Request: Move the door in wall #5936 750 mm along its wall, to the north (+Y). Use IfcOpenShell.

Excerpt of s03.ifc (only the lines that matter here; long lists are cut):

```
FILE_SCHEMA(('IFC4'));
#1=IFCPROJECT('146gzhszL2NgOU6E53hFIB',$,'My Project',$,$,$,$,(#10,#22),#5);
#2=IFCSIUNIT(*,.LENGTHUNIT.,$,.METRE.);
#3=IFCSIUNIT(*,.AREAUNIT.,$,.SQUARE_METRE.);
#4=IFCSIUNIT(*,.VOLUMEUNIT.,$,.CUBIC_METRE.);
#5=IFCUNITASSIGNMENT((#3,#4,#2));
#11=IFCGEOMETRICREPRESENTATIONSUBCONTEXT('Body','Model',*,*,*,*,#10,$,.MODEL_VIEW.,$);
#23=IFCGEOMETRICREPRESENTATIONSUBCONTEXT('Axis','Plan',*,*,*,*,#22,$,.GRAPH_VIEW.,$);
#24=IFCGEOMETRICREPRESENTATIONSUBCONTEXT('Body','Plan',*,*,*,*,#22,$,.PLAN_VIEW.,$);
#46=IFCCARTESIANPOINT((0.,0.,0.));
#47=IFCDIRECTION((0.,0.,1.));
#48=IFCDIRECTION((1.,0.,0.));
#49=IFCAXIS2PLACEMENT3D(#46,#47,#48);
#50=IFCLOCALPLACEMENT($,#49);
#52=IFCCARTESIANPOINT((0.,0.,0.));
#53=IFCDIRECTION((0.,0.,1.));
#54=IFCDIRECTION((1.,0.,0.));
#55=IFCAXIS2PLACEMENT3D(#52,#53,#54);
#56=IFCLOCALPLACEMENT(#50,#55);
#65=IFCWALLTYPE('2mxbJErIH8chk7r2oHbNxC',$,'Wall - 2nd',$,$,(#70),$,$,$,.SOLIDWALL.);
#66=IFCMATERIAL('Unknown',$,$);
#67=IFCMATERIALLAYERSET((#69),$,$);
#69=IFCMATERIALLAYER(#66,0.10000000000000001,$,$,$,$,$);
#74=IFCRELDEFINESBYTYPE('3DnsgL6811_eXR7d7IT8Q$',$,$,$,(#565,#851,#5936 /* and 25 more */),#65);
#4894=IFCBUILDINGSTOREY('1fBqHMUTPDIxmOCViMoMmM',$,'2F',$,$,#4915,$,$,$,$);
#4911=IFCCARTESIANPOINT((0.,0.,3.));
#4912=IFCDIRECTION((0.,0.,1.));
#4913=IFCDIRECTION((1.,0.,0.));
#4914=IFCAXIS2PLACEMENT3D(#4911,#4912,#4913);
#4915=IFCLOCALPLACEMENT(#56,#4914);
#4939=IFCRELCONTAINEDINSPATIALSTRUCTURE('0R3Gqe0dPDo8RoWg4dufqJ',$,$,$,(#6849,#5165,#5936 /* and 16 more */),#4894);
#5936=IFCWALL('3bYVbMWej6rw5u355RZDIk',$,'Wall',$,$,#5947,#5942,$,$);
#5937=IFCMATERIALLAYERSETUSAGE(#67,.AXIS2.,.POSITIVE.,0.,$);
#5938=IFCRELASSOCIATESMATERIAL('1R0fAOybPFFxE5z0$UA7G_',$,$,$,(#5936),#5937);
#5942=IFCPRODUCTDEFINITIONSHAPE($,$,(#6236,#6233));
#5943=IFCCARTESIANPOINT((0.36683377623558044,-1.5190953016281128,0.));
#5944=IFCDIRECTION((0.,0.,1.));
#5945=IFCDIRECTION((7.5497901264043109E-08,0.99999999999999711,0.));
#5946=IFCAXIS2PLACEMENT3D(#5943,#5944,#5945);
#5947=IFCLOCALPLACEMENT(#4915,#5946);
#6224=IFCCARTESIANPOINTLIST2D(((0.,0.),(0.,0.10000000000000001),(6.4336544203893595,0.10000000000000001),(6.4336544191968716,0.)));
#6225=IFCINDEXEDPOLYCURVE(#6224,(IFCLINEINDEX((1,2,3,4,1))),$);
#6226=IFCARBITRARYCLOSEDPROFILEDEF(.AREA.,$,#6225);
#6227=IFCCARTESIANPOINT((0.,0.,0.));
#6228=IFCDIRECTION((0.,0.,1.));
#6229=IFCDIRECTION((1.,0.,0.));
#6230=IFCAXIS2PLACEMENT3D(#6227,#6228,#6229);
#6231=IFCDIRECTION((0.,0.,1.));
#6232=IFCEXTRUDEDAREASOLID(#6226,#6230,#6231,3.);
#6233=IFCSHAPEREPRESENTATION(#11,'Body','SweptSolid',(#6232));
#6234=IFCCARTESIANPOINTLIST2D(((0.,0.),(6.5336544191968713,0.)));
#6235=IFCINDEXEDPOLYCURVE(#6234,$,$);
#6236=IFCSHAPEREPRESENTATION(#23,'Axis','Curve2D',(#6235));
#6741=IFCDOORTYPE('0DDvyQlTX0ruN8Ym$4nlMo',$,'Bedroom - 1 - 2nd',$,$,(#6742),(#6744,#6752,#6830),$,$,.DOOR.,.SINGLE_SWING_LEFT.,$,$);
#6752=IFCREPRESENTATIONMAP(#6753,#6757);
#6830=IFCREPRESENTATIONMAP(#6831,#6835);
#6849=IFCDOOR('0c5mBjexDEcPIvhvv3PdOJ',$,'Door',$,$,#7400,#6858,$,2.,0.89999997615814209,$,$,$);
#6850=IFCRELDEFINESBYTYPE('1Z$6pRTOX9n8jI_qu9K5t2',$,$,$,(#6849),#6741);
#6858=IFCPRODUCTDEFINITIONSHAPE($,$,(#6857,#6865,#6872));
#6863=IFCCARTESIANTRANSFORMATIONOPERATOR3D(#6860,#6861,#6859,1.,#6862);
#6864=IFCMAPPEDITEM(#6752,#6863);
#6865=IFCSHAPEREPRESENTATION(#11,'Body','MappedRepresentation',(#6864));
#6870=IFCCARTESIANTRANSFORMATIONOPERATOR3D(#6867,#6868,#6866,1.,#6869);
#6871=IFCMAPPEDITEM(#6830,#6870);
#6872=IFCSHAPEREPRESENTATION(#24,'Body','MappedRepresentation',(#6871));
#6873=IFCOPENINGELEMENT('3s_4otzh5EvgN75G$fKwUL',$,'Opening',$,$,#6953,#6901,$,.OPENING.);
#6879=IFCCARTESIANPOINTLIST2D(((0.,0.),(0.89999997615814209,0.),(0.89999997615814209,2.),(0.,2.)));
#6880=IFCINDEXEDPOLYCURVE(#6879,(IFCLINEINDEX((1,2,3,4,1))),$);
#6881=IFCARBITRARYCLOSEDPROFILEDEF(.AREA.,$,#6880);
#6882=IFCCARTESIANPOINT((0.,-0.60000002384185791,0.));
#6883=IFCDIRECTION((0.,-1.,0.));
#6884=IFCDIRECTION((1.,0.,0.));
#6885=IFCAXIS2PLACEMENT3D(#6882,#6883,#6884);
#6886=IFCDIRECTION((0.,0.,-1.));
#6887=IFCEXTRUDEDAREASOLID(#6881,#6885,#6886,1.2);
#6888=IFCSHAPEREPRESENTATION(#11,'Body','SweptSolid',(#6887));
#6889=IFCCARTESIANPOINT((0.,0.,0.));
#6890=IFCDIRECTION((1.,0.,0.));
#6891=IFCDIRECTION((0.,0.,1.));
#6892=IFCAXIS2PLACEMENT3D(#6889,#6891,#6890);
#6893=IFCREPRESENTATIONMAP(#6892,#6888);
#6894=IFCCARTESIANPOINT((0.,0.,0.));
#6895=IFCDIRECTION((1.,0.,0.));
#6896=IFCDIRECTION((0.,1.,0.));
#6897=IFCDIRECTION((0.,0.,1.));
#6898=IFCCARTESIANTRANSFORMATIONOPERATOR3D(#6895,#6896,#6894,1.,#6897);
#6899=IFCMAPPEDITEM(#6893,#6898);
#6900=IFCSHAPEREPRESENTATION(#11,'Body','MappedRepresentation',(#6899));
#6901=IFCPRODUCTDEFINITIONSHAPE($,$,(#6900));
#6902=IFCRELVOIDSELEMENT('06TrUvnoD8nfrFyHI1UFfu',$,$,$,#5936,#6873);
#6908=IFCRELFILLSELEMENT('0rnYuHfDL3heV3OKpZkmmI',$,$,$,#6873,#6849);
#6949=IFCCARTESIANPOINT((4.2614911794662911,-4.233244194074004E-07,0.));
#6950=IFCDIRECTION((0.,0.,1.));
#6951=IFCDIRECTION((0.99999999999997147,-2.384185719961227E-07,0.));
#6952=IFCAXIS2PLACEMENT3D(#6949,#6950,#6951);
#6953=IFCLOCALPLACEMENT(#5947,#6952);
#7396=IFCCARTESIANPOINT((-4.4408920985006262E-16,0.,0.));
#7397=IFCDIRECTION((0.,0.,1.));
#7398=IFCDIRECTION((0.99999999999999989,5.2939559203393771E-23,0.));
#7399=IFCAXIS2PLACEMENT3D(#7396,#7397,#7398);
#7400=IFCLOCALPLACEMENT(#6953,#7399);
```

```python
import ifcopenshell
import ifcopenshell.api.geometry
import ifcopenshell.util.placement
import ifcopenshell.util.unit

model = ifcopenshell.open("s03.ifc")
unit_scale = ifcopenshell.util.unit.calculate_unit_scale(model)

door = model.by_guid("0c5mBjexDEcPIvhvv3PdOJ")
opening = door.FillsVoids[0].RelatingOpeningElement
wall = opening.VoidsElements[0].RelatingBuildingElement

wall_matrix = ifcopenshell.util.placement.get_local_placement(wall.ObjectPlacement)
shift = wall_matrix[:3, 0] * 0.75 / unit_scale
before = ifcopenshell.util.placement.get_local_placement(door.ObjectPlacement)[:3, 3].copy()

# The door is placed relative to its opening, so it follows when the opening moves.
matrix = ifcopenshell.util.placement.get_local_placement(opening.ObjectPlacement)
matrix[:3, 3] += shift
ifcopenshell.api.geometry.edit_object_placement(
    model, product=opening, matrix=matrix, is_si=False, should_transform_children=True
)

after = ifcopenshell.util.placement.get_local_placement(door.ObjectPlacement)[:3, 3]
print("door moved by", (after - before).round(3) + 0.0)

model.write("s03_edited.ifc")
```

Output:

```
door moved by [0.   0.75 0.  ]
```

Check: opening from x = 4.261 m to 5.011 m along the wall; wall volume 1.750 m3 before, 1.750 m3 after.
